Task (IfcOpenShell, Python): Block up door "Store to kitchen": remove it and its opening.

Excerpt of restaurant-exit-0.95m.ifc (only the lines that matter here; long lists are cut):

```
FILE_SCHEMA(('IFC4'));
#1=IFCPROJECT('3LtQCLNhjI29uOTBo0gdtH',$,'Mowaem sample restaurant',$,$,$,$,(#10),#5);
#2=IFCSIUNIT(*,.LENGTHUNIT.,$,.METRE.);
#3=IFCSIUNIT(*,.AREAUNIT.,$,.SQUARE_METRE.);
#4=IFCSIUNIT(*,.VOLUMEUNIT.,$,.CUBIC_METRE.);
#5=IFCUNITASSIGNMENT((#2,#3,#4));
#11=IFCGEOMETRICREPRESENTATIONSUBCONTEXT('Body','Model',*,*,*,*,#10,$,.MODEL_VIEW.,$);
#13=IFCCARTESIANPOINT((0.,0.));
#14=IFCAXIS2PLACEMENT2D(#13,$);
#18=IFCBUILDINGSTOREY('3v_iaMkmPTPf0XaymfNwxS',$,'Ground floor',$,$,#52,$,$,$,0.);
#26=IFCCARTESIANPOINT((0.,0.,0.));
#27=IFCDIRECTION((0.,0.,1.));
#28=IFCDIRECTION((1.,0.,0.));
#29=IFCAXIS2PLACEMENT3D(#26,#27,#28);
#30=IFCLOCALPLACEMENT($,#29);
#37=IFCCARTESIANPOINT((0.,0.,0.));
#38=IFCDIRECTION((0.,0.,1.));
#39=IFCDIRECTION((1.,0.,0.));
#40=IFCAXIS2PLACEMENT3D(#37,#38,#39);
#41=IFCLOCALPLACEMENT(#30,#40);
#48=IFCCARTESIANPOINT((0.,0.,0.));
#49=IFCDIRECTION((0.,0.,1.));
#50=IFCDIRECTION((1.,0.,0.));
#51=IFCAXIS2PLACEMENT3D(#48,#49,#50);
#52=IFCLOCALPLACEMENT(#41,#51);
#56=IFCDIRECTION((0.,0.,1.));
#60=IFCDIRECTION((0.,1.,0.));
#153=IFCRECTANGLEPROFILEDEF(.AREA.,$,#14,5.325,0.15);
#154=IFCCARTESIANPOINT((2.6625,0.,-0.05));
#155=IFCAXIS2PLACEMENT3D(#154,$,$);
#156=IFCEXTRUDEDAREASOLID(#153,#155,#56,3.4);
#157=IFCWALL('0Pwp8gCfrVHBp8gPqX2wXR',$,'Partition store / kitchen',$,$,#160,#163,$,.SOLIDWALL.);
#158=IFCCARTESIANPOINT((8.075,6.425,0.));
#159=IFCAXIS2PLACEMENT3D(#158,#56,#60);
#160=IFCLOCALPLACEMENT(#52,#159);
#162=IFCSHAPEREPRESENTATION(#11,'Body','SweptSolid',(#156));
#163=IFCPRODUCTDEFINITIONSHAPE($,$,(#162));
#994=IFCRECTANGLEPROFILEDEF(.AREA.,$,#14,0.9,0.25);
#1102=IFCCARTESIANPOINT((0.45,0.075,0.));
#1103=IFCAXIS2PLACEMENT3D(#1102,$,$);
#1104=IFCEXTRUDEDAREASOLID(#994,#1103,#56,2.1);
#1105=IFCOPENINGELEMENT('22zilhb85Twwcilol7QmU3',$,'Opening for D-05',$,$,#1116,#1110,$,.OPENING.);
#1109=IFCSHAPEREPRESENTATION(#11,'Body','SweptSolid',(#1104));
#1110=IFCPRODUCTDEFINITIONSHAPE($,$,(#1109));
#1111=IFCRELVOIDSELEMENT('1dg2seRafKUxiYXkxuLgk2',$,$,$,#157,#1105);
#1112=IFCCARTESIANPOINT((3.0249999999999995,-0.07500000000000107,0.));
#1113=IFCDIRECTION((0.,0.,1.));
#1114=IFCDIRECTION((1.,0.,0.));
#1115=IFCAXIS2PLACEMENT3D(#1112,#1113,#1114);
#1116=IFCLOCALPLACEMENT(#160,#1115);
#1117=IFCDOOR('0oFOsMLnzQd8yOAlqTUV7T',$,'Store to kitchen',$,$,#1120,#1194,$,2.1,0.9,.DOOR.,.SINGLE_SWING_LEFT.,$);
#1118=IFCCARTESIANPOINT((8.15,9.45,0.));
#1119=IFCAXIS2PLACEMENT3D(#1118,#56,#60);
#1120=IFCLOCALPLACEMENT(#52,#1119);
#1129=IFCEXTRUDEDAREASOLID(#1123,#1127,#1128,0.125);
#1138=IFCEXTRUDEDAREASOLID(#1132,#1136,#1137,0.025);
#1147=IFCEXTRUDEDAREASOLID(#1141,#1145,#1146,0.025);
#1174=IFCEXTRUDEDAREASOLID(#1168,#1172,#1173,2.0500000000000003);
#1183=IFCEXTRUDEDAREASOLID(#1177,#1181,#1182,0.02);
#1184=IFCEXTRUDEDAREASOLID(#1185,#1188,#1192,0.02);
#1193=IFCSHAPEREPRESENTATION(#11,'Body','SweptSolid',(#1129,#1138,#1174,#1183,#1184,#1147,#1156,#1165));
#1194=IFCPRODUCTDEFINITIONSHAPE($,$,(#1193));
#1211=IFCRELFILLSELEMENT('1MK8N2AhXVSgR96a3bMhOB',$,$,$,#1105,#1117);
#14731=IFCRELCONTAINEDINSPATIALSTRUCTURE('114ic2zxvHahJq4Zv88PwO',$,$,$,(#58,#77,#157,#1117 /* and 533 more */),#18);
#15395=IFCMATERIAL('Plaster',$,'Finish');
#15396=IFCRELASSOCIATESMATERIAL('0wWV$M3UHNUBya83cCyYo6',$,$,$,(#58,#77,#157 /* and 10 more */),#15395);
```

```python
import ifcopenshell
import ifcopenshell.api.feature
import ifcopenshell.api.root
import ifcopenshell.geom
import ifcopenshell.util.shape

model = ifcopenshell.open("restaurant-exit-0.95m.ifc")
settings = ifcopenshell.geom.settings()


def volume(element):
    """Net volume in cubic metres, openings subtracted."""
    shape = ifcopenshell.geom.create_shape(settings, element)
    return ifcopenshell.util.shape.get_volume(shape.geometry)


door = model.by_guid("0oFOsMLnzQd8yOAlqTUV7T")
opening = door.FillsVoids[0].RelatingOpeningElement
wall = opening.VoidsElements[0].RelatingBuildingElement
before = volume(wall)

ifcopenshell.api.root.remove_product(model, product=door)
ifcopenshell.api.feature.remove_feature(model, feature=opening)

after = volume(wall)

print(f"wall volume {before:.3f} -> {after:.3f} m3")

model.write("restaurant-exit-0.95m_rev.ifc")
```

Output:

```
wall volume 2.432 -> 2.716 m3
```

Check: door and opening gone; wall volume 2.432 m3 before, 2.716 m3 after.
